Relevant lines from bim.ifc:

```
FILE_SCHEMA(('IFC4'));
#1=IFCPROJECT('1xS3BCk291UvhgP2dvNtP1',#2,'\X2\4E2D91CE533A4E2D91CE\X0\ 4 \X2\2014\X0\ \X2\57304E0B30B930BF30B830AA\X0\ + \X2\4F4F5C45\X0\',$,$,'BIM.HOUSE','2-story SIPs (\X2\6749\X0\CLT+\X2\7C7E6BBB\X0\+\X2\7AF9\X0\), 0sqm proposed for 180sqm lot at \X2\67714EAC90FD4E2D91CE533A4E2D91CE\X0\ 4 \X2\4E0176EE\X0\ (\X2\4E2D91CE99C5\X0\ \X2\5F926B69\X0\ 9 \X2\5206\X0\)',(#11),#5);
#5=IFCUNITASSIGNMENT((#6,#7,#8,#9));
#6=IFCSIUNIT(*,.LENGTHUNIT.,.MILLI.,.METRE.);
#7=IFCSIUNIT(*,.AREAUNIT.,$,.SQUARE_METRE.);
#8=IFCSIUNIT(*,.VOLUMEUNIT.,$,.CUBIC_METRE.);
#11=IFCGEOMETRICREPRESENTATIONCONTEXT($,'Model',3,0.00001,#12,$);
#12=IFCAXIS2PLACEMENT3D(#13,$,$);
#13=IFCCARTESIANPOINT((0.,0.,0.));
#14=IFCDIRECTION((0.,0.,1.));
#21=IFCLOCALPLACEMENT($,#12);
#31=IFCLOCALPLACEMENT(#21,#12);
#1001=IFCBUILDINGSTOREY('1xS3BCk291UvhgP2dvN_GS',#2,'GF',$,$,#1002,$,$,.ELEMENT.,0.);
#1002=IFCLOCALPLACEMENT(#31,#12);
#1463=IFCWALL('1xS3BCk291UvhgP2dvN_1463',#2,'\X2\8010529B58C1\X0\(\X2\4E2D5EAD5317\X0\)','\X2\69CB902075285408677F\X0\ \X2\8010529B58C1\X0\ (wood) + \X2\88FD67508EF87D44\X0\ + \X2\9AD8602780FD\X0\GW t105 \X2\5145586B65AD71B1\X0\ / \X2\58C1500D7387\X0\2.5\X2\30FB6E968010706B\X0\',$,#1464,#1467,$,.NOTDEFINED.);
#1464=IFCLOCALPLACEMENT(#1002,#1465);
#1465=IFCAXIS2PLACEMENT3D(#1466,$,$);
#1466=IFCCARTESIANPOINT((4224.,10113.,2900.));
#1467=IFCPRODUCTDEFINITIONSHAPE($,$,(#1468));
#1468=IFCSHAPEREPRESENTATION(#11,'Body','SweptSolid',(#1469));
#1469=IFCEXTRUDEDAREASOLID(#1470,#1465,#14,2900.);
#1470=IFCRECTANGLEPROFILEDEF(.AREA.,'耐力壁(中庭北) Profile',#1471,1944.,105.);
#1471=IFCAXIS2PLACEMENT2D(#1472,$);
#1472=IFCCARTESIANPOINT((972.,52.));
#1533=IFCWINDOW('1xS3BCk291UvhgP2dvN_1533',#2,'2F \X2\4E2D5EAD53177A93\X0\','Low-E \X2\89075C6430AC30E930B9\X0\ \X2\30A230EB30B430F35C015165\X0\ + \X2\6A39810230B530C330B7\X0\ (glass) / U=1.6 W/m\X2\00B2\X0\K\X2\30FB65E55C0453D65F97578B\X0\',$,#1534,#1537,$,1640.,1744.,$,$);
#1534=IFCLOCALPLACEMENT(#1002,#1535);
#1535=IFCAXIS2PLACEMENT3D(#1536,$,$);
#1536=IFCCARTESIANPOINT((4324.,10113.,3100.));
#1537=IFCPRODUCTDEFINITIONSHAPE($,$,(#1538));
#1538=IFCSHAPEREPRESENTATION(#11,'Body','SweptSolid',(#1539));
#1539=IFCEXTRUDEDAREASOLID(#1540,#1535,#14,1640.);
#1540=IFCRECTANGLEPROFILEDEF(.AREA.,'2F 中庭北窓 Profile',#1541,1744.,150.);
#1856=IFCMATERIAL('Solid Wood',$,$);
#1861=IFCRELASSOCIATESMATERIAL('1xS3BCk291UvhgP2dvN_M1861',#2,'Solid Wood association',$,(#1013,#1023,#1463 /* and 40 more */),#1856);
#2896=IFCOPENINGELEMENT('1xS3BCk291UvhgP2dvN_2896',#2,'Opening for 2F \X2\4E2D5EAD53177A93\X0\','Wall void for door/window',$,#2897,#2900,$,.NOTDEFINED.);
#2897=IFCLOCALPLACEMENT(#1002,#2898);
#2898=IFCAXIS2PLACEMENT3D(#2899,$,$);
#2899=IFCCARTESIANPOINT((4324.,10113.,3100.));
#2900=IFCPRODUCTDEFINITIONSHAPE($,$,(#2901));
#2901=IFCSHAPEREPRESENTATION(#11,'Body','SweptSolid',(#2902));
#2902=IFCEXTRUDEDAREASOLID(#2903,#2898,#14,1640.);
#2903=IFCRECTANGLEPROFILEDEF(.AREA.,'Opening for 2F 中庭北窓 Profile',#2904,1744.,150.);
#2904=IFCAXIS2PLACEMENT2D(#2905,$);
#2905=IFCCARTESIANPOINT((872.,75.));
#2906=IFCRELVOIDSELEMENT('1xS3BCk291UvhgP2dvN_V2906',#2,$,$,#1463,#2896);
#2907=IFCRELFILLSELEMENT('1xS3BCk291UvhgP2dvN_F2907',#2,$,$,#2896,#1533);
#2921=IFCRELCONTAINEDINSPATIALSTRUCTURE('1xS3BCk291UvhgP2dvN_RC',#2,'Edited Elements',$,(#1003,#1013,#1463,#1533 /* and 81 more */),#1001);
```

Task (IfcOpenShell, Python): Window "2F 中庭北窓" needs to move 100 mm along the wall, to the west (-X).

```python
import ifcopenshell
import ifcopenshell.api.geometry
import ifcopenshell.util.placement
import ifcopenshell.util.unit

model = ifcopenshell.open("bim.ifc")
unit_scale = ifcopenshell.util.unit.calculate_unit_scale(model)

window = model.by_guid("1xS3BCk291UvhgP2dvN_1533")
opening = window.FillsVoids[0].RelatingOpeningElement
wall = opening.VoidsElements[0].RelatingBuildingElement

wall_matrix = ifcopenshell.util.placement.get_local_placement(wall.ObjectPlacement)
shift = wall_matrix[:3, 0] * -0.1 / unit_scale
before = ifcopenshell.util.placement.get_local_placement(window.ObjectPlacement)[:3, 3].copy()

# The window is not placed relative to its opening, so move both.
for product in (opening, window):
    matrix = ifcopenshell.util.placement.get_local_placement(product.ObjectPlacement)
    matrix[:3, 3] += shift
    ifcopenshell.api.geometry.edit_object_placement(model, product=product, matrix=matrix, is_si=False)

after = ifcopenshell.util.placement.get_local_placement(window.ObjectPlacement)[:3, 3]
print("window moved by", (after - before).round(3) + 0.0)

model.write("bim_edited.ifc")
```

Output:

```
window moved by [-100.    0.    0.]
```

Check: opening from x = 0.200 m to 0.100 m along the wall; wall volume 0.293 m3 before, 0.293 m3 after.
